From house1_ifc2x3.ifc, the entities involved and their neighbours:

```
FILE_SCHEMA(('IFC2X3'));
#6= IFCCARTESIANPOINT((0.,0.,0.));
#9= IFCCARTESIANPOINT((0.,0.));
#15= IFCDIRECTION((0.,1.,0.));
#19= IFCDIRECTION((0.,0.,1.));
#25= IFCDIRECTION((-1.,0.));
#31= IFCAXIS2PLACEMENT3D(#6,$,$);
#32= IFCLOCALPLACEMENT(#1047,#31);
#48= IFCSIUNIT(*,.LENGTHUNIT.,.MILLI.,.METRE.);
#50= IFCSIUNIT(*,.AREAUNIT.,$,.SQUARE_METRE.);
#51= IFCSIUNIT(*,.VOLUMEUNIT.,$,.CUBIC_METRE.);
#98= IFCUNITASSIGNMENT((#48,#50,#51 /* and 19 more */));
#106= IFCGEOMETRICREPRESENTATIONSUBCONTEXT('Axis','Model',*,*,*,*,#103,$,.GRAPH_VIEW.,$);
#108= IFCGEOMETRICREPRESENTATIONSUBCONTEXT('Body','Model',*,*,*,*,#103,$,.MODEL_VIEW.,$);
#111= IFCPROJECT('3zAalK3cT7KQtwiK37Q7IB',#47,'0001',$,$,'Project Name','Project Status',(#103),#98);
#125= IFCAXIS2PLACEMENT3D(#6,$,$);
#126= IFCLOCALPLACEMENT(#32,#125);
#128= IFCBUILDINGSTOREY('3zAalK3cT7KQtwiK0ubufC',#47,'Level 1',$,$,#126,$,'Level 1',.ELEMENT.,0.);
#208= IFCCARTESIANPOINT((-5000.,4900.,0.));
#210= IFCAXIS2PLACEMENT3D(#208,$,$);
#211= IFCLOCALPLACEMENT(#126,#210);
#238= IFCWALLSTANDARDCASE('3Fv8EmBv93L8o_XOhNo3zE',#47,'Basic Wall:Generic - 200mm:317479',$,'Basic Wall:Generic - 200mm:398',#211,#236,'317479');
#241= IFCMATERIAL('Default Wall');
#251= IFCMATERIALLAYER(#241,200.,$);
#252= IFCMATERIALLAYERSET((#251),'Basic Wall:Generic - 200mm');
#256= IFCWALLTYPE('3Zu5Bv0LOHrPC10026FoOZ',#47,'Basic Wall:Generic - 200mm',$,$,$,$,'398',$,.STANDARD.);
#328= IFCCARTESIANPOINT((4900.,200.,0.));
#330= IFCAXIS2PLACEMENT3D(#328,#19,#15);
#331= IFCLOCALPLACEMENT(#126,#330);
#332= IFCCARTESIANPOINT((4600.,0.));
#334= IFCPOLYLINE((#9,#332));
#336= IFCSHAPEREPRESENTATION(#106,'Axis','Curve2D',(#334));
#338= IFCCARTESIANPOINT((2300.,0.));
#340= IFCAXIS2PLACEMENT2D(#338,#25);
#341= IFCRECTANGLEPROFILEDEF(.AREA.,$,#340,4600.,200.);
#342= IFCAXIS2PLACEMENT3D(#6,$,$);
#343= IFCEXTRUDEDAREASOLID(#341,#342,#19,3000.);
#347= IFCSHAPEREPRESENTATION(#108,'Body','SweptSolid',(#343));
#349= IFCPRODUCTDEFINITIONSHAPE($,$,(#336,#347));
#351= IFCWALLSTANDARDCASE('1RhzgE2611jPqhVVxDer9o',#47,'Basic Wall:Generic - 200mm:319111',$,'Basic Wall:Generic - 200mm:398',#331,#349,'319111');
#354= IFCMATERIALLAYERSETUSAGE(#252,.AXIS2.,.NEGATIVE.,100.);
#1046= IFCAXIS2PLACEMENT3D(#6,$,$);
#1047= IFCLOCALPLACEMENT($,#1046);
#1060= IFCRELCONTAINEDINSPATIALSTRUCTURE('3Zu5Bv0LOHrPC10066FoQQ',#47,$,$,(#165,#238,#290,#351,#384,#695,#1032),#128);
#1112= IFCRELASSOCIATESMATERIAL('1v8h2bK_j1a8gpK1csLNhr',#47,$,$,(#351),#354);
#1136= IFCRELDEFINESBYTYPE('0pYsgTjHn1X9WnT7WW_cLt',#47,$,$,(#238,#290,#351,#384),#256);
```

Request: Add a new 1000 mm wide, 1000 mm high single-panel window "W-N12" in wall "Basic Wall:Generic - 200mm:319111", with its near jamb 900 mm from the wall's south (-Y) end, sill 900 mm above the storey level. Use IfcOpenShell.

```python
import numpy as np
import ifcopenshell
import ifcopenshell.api.feature
import ifcopenshell.api.geometry
import ifcopenshell.api.root
import ifcopenshell.api.spatial
import ifcopenshell.api.type
import ifcopenshell.geom
import ifcopenshell.util.element
import ifcopenshell.util.placement
import ifcopenshell.util.representation
import ifcopenshell.util.shape
import ifcopenshell.util.unit

model = ifcopenshell.open("house1_ifc2x3.ifc")
unit_scale = ifcopenshell.util.unit.calculate_unit_scale(model)
settings = ifcopenshell.geom.settings()


def volume(element):
    """Net volume in cubic metres, openings subtracted."""
    shape = ifcopenshell.geom.create_shape(settings, element)
    return ifcopenshell.util.shape.get_volume(shape.geometry)


wall = model.by_guid("1RhzgE2611jPqhVVxDer9o")
storey = ifcopenshell.util.element.get_container(wall, ifc_class="IfcBuildingStorey")
context = ifcopenshell.util.representation.get_context(model, "Model", "Body", "MODEL_VIEW")
before = volume(wall)

width, height, from_end, sill = 1, 1, 0.9, 0.9  # metres

# The wall runs along its own X axis, and the end named is its -X end.
wall_shape = ifcopenshell.geom.create_shape(settings, wall)
x, y, z = ifcopenshell.util.shape.get_vertices(wall_shape.geometry).T
start = x.min() + from_end
face, thickness = float(y.min()), float(y.max() - y.min())
wall_matrix = ifcopenshell.util.placement.get_local_placement(wall.ObjectPlacement)
level = ifcopenshell.util.placement.get_local_placement(storey.ObjectPlacement)[2, 3]


def in_wall(x, y):
    """Placement at x, y metres in the wall's axes, at sill height."""
    matrix = wall_matrix.copy()
    matrix[:, 3] = wall_matrix @ np.array([x / unit_scale, y / unit_scale, 0.0, 1.0])
    matrix[2, 3] = level + sill / unit_scale
    return matrix


# Opening: a box that overshoots both wall faces by 50 mm.
opening = ifcopenshell.api.root.create_entity(model, ifc_class="IfcOpeningElement")
box = ifcopenshell.api.geometry.add_wall_representation(
    model, context=context, length=width, height=height, thickness=thickness + 0.1
)
ifcopenshell.api.geometry.assign_representation(model, product=opening, representation=box)
ifcopenshell.api.geometry.edit_object_placement(model, product=opening, matrix=in_wall(start, face - 0.05), is_si=False)
ifcopenshell.api.feature.add_feature(model, feature=opening, element=wall)

window = ifcopenshell.api.root.create_entity(model, ifc_class="IfcWindow", name="W-N12")
window.OverallWidth, window.OverallHeight = width / unit_scale, height / unit_scale
body = ifcopenshell.api.geometry.add_window_representation(
    model,
    context=context,
    overall_width=window.OverallWidth,
    overall_height=window.OverallHeight,
    partition_type="SINGLE_PANEL",
)
ifcopenshell.api.geometry.assign_representation(model, product=window, representation=body)
ifcopenshell.api.spatial.assign_container(model, products=[window], relating_structure=storey)
fills = ifcopenshell.api.feature.add_filling(model, opening=opening, element=window)
fills.OwnerHistory = window.OwnerHistory  # required in IFC2X3

# IFC2X3 keeps the operation on the window style.
style = ifcopenshell.api.root.create_entity(model, ifc_class="IfcWindowStyle", name="W-N12")
style.OperationType, style.ConstructionType = "SINGLE_PANEL", "NOTDEFINED"
style.ParameterTakesPrecedence = style.Sizeable = False
ifcopenshell.api.type.assign_type(model, related_objects=[window], relating_type=style)

# Centre the window in the wall's thickness.
ifcopenshell.api.geometry.edit_object_placement(model, product=window, matrix=in_wall(start, face), is_si=False)
window_shape = ifcopenshell.geom.create_shape(settings, window)
depth = ifcopenshell.util.shape.get_vertices(window_shape.geometry)[:, 1]
offset = face + thickness / 2 - (depth.min() + depth.max()) / 2
ifcopenshell.api.geometry.edit_object_placement(model, product=window, matrix=in_wall(start, offset), is_si=False)

after = volume(wall)

print(f"wall volume {before:.3f} -> {after:.3f} m3")

model.write("house1_ifc2x3_updated.ifc")
```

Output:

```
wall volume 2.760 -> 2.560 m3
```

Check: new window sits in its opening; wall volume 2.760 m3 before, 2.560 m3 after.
